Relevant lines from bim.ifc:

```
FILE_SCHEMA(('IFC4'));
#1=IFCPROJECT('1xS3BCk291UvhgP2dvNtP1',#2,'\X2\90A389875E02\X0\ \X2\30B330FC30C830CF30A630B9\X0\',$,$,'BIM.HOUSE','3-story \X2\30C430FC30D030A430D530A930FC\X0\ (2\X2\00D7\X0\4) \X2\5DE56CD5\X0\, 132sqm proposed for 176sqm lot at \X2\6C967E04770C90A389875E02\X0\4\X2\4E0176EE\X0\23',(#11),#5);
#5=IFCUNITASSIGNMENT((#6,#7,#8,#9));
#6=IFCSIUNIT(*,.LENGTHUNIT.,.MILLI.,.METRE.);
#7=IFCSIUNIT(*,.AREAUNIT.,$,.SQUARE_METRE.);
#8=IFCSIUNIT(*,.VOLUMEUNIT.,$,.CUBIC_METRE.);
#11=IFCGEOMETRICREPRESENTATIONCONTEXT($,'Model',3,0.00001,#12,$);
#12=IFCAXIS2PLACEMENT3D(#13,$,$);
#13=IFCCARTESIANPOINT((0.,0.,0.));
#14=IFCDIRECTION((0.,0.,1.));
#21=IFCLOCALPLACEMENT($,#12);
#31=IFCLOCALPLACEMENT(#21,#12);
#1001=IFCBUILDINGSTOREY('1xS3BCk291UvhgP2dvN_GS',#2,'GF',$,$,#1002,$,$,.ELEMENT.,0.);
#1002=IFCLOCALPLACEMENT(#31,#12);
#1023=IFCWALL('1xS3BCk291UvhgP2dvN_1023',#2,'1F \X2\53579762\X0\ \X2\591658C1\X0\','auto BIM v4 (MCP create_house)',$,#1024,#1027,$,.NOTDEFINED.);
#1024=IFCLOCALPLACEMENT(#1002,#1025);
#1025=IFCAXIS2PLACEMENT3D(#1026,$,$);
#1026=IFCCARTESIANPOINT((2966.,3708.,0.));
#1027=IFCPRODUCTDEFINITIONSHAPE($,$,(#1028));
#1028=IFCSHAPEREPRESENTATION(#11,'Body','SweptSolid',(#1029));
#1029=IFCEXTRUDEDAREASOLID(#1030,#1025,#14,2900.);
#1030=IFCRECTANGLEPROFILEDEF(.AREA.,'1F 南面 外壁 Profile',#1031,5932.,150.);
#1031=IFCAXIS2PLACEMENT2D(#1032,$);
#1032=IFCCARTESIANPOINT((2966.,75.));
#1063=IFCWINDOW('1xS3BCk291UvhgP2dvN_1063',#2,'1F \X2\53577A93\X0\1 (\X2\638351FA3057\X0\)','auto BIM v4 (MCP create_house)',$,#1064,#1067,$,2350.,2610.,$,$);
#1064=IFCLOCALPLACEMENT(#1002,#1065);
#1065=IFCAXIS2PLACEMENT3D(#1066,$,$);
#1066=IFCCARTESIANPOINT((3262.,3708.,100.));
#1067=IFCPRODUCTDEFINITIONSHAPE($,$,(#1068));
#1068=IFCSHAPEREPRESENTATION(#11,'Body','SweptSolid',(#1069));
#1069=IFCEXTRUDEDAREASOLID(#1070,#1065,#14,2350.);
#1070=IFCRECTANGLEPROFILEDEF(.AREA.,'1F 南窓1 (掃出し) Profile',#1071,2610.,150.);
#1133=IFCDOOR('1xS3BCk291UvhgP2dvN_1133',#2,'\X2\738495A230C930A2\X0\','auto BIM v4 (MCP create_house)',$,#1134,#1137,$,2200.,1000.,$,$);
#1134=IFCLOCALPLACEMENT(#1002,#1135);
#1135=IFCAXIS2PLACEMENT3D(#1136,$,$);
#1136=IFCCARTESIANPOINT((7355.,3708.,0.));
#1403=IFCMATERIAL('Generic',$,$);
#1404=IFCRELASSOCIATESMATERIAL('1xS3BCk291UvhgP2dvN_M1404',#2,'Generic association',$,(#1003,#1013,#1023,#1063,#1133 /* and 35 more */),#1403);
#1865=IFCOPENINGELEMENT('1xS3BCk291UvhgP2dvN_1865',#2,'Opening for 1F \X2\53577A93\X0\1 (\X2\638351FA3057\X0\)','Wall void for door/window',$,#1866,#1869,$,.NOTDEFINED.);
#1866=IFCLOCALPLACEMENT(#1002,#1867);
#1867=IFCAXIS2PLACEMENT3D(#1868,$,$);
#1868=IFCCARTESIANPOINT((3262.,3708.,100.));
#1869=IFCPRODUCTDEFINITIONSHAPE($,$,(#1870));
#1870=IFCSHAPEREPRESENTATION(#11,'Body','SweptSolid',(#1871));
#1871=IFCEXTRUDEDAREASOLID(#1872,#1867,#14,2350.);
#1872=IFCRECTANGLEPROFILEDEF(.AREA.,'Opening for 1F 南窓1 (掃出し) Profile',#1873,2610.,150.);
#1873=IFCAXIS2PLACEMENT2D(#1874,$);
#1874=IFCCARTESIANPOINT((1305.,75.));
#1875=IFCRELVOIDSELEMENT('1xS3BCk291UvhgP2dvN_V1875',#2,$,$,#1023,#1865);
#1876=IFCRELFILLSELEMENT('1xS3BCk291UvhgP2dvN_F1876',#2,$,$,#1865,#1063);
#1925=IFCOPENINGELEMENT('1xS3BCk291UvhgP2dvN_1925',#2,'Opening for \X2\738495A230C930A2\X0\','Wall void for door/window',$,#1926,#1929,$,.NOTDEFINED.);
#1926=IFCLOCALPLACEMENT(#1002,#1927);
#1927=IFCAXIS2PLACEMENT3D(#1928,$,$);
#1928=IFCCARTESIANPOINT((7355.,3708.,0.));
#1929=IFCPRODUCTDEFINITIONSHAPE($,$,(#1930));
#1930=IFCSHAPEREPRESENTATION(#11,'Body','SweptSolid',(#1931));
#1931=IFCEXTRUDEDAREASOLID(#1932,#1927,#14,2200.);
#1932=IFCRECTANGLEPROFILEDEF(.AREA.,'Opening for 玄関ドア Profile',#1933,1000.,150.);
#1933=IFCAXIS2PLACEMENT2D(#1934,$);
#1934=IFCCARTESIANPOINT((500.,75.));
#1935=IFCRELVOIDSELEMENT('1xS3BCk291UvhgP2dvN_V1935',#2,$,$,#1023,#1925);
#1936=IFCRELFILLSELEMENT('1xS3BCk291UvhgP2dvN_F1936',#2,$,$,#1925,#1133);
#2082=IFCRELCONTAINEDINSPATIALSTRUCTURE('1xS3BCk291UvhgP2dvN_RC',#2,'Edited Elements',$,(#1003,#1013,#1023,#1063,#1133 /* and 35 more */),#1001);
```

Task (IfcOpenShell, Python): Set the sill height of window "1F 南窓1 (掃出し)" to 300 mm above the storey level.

```python
import numpy as np
import ifcopenshell
import ifcopenshell.api.geometry
import ifcopenshell.geom
import ifcopenshell.util.element
import ifcopenshell.util.placement
import ifcopenshell.util.shape
import ifcopenshell.util.unit

model = ifcopenshell.open("bim.ifc")
unit_scale = ifcopenshell.util.unit.calculate_unit_scale(model)

window = model.by_id(1063)
opening = window.FillsVoids[0].RelatingOpeningElement
storey = ifcopenshell.util.element.get_container(window, ifc_class="IfcBuildingStorey")
level = ifcopenshell.util.placement.get_local_placement(storey.ObjectPlacement)[2, 3]

# The opening's origin need not be at the sill, so measure its lowest point.
shape = ifcopenshell.geom.create_shape(ifcopenshell.geom.settings(), opening)
bottom = ifcopenshell.util.shape.get_shape_bottom_elevation(shape, shape.geometry) / unit_scale
dz = level + 300.0 - bottom

shift = np.array([0.0, 0.0, dz])
# The window is not placed relative to its opening, so move both.
for product in (opening, window):
    matrix = ifcopenshell.util.placement.get_local_placement(product.ObjectPlacement)
    matrix[:3, 3] += shift
    ifcopenshell.api.geometry.edit_object_placement(model, product=product, matrix=matrix, is_si=False)

print(f"moved by {dz * unit_scale:+.3f} m")

model.write("bim_edited.ifc")
```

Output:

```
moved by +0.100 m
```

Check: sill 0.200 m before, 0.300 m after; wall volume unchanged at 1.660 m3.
